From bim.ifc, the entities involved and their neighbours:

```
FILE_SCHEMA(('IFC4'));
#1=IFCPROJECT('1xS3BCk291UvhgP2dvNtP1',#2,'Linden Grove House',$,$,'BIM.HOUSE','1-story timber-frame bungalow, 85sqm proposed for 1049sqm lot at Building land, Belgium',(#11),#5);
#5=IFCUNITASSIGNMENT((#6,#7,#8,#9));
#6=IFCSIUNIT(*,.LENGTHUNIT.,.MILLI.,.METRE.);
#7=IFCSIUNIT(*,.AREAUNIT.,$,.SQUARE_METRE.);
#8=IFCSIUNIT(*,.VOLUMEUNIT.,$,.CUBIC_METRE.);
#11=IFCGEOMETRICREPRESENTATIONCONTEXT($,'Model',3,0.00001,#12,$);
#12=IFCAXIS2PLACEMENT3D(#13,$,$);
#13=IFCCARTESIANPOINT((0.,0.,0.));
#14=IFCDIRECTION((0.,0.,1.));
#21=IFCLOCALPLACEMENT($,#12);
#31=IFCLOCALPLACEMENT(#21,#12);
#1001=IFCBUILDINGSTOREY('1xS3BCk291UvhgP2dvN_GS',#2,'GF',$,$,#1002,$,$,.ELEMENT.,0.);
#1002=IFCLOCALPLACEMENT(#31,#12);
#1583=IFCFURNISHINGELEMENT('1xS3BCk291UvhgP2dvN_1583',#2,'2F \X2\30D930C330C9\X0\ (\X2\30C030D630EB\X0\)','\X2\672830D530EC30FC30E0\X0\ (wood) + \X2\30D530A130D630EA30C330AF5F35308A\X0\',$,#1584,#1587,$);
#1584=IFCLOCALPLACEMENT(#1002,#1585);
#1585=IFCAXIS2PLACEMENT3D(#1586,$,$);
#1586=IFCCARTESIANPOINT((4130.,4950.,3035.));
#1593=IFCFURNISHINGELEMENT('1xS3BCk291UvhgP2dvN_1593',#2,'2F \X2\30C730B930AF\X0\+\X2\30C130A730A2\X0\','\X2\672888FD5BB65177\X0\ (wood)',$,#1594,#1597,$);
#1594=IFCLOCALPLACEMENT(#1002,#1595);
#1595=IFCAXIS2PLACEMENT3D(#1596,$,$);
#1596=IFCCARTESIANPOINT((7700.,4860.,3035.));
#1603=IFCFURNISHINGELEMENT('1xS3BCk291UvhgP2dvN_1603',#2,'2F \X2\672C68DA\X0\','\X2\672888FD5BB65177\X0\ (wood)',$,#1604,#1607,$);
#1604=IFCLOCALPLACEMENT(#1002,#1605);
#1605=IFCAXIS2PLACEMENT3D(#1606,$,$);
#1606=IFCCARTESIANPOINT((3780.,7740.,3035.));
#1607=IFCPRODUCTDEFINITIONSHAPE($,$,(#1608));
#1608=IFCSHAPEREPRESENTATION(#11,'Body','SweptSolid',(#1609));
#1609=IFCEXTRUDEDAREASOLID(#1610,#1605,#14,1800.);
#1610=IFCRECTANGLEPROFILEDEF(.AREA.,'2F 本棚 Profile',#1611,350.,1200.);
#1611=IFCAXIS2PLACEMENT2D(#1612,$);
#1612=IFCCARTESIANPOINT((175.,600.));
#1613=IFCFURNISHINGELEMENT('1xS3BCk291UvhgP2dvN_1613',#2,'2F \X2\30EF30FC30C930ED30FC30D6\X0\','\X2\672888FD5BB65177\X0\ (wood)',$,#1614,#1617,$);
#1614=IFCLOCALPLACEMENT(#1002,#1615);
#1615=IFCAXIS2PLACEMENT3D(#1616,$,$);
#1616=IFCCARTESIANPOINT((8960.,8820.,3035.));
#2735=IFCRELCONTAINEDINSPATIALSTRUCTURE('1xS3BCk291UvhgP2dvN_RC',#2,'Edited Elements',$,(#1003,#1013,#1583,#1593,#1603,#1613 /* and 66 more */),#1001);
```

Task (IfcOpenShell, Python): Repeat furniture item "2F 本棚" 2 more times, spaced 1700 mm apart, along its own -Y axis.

```python
import ifcopenshell
import ifcopenshell.api.geometry
import ifcopenshell.api.root
import ifcopenshell.util.element
import ifcopenshell.util.placement

model = ifcopenshell.open("bim.ifc")


def reuse_history(source, copy):
    """copy_class also copies each property set's owner history, people and application; keep the originals."""
    for rel in copy.IsDefinedBy:
        if rel.is_a("IfcRelDefinesByProperties") and (history := rel.RelatingPropertyDefinition.OwnerHistory):
            rel.RelatingPropertyDefinition.OwnerHistory = source.OwnerHistory
            ifcopenshell.util.element.remove_deep2(model, history)


source = model.by_guid("1xS3BCk291UvhgP2dvN_1603")
base = ifcopenshell.util.placement.get_local_placement(source.ObjectPlacement)
step = -base[:3, 1] * 1700.0

for i in range(1, 3):
    copy = ifcopenshell.api.root.copy_class(model, product=source)
    copy.Representation = ifcopenshell.util.element.copy_deep(
        model, source.Representation, exclude=["IfcGeometricRepresentationContext", "IfcRepresentationMap"]
    )
    reuse_history(source, copy)
    matrix = base.copy()
    matrix[:3, 3] += i * step
    print("added at", matrix[:3, 3].round(3) + 0.0)
    ifcopenshell.api.geometry.edit_object_placement(model, product=copy, matrix=matrix, is_si=False)

model.write("bim-out.ifc")
```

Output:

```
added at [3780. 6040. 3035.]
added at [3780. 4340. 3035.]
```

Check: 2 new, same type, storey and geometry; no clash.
